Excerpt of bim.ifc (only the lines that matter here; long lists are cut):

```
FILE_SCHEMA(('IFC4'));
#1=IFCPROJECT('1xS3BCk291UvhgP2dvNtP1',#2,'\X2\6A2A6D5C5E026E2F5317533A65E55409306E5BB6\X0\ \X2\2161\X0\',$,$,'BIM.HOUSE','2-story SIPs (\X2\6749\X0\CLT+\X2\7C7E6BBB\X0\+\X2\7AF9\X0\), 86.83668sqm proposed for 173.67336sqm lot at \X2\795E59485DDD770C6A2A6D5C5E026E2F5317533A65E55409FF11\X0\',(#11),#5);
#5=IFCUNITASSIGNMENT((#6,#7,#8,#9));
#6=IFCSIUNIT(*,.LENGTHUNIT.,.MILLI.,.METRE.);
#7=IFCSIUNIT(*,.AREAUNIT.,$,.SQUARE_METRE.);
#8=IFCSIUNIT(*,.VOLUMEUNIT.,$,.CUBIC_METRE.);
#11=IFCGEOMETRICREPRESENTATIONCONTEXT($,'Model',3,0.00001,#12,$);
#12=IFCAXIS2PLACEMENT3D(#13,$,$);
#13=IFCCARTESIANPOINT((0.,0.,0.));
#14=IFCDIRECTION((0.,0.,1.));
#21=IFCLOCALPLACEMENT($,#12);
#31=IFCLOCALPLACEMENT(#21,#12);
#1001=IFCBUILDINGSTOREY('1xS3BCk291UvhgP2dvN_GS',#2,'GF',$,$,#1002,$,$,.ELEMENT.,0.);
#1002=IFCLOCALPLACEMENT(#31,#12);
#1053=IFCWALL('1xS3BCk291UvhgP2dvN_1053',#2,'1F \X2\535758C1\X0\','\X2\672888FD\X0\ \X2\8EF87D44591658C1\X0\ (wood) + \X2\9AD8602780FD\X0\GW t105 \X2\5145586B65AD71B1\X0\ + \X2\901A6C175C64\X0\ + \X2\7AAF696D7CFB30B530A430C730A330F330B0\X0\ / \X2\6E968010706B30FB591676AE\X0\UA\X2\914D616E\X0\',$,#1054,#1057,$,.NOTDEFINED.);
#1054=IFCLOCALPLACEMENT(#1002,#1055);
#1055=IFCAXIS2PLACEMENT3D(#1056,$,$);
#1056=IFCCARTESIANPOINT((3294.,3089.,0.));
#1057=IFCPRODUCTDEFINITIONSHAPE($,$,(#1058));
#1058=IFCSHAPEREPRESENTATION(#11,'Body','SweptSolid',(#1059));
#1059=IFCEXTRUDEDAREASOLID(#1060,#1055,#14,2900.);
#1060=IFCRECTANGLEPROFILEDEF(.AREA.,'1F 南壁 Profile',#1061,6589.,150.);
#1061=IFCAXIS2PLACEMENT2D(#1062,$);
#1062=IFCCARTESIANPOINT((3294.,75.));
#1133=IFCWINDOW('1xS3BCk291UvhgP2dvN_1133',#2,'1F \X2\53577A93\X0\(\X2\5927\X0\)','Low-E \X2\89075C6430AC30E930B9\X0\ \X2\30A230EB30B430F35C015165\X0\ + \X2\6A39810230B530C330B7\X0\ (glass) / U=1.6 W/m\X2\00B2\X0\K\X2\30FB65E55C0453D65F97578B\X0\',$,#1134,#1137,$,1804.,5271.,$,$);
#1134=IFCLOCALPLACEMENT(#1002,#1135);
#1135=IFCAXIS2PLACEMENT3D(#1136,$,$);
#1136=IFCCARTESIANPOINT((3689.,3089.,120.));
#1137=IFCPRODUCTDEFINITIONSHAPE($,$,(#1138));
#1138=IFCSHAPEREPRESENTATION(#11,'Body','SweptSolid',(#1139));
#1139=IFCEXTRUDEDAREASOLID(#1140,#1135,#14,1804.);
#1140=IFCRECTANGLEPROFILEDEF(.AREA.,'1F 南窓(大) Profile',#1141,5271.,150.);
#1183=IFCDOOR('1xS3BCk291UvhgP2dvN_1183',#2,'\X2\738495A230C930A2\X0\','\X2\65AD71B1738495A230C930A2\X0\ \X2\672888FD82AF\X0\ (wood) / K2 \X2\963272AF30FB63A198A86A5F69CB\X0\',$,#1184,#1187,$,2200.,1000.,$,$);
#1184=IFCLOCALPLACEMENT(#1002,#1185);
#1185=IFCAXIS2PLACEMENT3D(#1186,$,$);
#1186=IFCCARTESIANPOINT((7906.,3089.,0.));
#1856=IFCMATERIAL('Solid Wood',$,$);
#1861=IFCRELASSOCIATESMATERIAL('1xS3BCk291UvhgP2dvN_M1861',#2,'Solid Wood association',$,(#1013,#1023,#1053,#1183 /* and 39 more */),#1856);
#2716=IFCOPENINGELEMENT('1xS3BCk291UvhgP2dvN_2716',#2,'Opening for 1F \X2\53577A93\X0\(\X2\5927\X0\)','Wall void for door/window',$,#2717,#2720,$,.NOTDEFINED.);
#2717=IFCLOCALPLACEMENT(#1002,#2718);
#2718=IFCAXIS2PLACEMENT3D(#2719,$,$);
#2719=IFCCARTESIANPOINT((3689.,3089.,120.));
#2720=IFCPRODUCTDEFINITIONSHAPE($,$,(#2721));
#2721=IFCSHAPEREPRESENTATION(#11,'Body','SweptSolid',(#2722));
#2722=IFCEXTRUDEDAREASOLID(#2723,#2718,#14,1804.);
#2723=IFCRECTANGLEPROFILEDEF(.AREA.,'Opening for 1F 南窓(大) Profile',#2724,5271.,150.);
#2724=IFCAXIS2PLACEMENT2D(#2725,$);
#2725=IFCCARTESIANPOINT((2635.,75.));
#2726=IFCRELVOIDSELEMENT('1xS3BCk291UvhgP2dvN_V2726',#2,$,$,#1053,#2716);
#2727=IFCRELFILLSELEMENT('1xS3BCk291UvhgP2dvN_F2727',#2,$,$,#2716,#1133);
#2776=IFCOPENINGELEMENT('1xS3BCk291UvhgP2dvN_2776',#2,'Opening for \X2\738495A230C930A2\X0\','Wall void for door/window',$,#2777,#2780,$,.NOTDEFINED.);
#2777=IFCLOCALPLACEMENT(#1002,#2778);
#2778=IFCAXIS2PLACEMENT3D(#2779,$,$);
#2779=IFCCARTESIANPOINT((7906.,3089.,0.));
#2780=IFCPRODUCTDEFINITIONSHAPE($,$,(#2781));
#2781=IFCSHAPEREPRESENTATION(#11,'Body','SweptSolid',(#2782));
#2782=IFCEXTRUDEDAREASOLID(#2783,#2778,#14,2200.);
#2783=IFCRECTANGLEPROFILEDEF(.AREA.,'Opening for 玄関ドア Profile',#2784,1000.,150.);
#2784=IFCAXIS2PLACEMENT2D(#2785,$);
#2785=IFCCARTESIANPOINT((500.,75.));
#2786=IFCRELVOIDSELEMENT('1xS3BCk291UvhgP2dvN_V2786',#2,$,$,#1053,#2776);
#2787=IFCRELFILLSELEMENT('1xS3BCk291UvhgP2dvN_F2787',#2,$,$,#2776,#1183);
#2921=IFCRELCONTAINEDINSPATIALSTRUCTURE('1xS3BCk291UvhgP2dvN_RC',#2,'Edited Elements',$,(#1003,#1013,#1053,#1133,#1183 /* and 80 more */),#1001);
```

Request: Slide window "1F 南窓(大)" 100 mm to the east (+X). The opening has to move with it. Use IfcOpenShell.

```python
import ifcopenshell
import ifcopenshell.api.geometry
import ifcopenshell.util.placement

model = ifcopenshell.open("bim.ifc")

window = model.by_guid("1xS3BCk291UvhgP2dvN_1133")
opening = window.FillsVoids[0].RelatingOpeningElement
wall = opening.VoidsElements[0].RelatingBuildingElement

wall_matrix = ifcopenshell.util.placement.get_local_placement(wall.ObjectPlacement)
shift = wall_matrix[:3, 0] * 100.0
before = ifcopenshell.util.placement.get_local_placement(window.ObjectPlacement)[:3, 3].copy()

# The window is not placed relative to its opening, so move both.
for product in (opening, window):
    matrix = ifcopenshell.util.placement.get_local_placement(product.ObjectPlacement)
    matrix[:3, 3] += shift
    ifcopenshell.api.geometry.edit_object_placement(model, product=product, matrix=matrix, is_si=False)

after = ifcopenshell.util.placement.get_local_placement(window.ObjectPlacement)[:3, 3]
print("window moved by", (after - before).round(3) + 0.0)

model.write("bim_edited.ifc")
```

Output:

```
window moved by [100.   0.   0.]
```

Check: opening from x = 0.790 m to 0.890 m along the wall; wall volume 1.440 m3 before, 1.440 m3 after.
